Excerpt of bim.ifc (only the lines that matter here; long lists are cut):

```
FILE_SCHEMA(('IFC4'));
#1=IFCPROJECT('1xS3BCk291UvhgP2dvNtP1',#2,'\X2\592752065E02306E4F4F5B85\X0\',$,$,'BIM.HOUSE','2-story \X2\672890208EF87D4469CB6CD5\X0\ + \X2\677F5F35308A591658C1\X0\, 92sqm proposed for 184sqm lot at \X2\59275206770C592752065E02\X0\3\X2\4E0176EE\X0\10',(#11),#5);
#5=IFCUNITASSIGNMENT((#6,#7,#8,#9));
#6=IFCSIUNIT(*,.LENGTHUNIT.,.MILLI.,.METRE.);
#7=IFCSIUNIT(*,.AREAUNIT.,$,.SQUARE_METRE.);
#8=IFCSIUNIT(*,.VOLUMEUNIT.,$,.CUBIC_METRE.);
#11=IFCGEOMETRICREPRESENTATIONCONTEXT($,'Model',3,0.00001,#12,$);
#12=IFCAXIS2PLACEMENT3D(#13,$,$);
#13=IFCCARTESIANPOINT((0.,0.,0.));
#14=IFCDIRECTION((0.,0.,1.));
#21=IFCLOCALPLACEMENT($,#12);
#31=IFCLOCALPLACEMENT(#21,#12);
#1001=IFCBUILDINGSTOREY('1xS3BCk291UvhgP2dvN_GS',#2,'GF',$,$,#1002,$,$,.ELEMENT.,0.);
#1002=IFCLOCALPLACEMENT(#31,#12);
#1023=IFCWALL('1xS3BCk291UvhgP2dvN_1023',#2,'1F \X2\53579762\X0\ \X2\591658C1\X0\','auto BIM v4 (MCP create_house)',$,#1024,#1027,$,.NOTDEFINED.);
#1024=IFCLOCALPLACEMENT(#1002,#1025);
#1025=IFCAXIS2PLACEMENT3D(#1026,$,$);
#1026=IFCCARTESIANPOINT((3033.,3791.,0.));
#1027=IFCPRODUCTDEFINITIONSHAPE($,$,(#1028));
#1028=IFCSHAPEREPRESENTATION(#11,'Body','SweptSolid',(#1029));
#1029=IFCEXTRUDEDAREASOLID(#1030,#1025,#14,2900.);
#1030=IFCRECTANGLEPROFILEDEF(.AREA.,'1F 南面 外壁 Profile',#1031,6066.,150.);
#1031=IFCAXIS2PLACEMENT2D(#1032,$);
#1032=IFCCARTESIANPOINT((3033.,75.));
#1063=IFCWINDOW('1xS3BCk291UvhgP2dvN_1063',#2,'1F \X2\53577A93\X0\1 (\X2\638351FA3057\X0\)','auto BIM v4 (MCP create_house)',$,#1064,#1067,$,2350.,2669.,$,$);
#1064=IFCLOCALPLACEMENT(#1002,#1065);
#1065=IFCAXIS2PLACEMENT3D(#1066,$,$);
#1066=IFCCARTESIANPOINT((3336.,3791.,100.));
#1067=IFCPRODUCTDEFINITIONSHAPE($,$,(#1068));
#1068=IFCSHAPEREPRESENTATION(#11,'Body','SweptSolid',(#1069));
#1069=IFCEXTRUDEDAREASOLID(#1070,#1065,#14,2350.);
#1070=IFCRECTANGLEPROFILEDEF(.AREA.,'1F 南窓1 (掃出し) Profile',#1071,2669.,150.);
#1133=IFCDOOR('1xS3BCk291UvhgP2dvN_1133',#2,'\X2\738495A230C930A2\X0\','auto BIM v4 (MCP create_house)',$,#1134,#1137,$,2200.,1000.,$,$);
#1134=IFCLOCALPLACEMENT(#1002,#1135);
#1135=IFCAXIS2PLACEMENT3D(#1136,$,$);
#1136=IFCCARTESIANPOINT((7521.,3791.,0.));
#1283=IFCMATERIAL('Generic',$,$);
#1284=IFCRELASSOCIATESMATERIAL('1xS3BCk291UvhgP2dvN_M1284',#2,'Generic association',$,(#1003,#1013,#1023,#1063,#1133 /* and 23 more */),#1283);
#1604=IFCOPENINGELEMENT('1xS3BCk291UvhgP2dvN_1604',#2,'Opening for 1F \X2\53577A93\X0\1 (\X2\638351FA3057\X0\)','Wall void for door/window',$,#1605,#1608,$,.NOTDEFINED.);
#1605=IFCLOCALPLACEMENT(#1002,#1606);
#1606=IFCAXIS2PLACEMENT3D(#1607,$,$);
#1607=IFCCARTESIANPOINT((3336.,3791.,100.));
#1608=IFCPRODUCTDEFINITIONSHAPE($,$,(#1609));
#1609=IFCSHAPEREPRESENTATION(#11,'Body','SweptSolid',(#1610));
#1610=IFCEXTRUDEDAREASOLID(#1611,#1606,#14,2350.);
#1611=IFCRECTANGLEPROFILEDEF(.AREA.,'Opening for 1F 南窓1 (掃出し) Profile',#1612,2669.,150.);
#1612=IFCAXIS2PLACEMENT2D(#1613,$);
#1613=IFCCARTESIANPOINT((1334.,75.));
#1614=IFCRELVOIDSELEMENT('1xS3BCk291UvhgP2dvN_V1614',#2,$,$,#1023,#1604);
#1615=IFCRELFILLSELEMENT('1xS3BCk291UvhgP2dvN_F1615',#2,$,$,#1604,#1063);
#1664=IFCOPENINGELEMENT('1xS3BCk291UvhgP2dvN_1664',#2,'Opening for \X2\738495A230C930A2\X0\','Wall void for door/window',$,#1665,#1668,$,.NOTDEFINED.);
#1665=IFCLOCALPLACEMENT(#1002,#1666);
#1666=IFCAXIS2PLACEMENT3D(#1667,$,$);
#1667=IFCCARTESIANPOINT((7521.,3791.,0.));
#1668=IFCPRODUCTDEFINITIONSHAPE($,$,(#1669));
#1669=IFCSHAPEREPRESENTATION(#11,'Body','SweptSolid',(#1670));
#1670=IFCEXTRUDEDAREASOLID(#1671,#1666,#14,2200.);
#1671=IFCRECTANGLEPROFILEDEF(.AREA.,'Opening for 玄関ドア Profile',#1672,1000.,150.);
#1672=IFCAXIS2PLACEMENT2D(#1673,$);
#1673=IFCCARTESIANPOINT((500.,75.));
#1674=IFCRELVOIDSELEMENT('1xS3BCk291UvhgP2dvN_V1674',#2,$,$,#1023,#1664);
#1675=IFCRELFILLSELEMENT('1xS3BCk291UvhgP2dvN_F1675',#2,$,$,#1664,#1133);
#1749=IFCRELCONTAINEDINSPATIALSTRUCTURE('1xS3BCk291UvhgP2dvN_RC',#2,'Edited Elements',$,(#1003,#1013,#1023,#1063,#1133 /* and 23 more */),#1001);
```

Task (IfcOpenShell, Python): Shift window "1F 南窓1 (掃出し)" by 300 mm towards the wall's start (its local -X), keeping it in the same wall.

```python
import ifcopenshell
import ifcopenshell.api.geometry
import ifcopenshell.util.placement

model = ifcopenshell.open("bim.ifc")

window = model.by_guid("1xS3BCk291UvhgP2dvN_1063")
opening = window.FillsVoids[0].RelatingOpeningElement
wall = opening.VoidsElements[0].RelatingBuildingElement

wall_matrix = ifcopenshell.util.placement.get_local_placement(wall.ObjectPlacement)
shift = wall_matrix[:3, 0] * -300.0
before = ifcopenshell.util.placement.get_local_placement(window.ObjectPlacement)[:3, 3].copy()

# The window is not placed relative to its opening, so move both.
for product in (opening, window):
    matrix = ifcopenshell.util.placement.get_local_placement(product.ObjectPlacement)
    matrix[:3, 3] += shift
    ifcopenshell.api.geometry.edit_object_placement(model, product=product, matrix=matrix, is_si=False)

after = ifcopenshell.util.placement.get_local_placement(window.ObjectPlacement)[:3, 3]
print("window moved by", (after - before).round(3) + 0.0)

model.write("bim_updated.ifc")
```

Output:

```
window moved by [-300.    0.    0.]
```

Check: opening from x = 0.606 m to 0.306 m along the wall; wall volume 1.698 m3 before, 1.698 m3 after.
